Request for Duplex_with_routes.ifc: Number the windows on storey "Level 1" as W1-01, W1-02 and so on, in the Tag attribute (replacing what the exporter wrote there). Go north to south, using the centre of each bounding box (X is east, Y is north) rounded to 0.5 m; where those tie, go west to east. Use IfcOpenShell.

First a look at what the model holds.

```python
import ifcopenshell
import ifcopenshell.util.element
import ifcopenshell.util.placement

model = ifcopenshell.open("Duplex_with_routes.ifc")
print(model.schema)
storey = next(s for s in model.by_type("IfcBuildingStorey") if s.Name == "Level 1")
windows = [e for e in ifcopenshell.util.element.get_decomposition(storey) if e.is_a("IfcWindow")]
for e in sorted(windows, key=lambda e: e.id()):
    origin = ifcopenshell.util.placement.get_local_placement(e.ObjectPlacement)[:3, 3]
    print(e.id(), e.Tag, e.Name, origin.round(2) + 0.0, sep=" | ")
```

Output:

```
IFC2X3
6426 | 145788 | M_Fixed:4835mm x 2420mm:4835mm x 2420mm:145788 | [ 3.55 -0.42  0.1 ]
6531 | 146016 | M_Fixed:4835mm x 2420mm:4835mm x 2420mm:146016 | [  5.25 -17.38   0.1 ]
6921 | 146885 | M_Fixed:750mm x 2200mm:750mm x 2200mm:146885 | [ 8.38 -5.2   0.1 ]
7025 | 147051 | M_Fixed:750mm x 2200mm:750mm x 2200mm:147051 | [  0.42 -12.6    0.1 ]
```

```python
import ifcopenshell
import ifcopenshell.geom
import ifcopenshell.util.element
import ifcopenshell.util.shape

model = ifcopenshell.open("Duplex_with_routes.ifc")
settings = ifcopenshell.geom.settings()
settings.set("use-world-coords", True)


def centre(element):
    shape = ifcopenshell.geom.create_shape(settings, element)
    return ifcopenshell.util.shape.get_bbox_centroid(shape.geometry)


storey = next(s for s in model.by_type("IfcBuildingStorey") if s.Name == "Level 1")
windows = [e for e in ifcopenshell.util.element.get_decomposition(storey) if e.is_a("IfcWindow")]

# Insertion points can sit at a corner or the storey origin, so sort by the geometry (in metres).
centres = {e: centre(e) for e in windows}
windows.sort(key=lambda e: (-round(centres[e][1] / 0.5), centres[e][0]))

for i, e in enumerate(windows, start=1):
    number = f"W1-{i:02d}"
    e.Tag = number
    print(e.id(), number)

model.write("Duplex_with_routes_rev.ifc")
```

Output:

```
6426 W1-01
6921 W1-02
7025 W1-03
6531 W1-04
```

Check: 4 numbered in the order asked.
